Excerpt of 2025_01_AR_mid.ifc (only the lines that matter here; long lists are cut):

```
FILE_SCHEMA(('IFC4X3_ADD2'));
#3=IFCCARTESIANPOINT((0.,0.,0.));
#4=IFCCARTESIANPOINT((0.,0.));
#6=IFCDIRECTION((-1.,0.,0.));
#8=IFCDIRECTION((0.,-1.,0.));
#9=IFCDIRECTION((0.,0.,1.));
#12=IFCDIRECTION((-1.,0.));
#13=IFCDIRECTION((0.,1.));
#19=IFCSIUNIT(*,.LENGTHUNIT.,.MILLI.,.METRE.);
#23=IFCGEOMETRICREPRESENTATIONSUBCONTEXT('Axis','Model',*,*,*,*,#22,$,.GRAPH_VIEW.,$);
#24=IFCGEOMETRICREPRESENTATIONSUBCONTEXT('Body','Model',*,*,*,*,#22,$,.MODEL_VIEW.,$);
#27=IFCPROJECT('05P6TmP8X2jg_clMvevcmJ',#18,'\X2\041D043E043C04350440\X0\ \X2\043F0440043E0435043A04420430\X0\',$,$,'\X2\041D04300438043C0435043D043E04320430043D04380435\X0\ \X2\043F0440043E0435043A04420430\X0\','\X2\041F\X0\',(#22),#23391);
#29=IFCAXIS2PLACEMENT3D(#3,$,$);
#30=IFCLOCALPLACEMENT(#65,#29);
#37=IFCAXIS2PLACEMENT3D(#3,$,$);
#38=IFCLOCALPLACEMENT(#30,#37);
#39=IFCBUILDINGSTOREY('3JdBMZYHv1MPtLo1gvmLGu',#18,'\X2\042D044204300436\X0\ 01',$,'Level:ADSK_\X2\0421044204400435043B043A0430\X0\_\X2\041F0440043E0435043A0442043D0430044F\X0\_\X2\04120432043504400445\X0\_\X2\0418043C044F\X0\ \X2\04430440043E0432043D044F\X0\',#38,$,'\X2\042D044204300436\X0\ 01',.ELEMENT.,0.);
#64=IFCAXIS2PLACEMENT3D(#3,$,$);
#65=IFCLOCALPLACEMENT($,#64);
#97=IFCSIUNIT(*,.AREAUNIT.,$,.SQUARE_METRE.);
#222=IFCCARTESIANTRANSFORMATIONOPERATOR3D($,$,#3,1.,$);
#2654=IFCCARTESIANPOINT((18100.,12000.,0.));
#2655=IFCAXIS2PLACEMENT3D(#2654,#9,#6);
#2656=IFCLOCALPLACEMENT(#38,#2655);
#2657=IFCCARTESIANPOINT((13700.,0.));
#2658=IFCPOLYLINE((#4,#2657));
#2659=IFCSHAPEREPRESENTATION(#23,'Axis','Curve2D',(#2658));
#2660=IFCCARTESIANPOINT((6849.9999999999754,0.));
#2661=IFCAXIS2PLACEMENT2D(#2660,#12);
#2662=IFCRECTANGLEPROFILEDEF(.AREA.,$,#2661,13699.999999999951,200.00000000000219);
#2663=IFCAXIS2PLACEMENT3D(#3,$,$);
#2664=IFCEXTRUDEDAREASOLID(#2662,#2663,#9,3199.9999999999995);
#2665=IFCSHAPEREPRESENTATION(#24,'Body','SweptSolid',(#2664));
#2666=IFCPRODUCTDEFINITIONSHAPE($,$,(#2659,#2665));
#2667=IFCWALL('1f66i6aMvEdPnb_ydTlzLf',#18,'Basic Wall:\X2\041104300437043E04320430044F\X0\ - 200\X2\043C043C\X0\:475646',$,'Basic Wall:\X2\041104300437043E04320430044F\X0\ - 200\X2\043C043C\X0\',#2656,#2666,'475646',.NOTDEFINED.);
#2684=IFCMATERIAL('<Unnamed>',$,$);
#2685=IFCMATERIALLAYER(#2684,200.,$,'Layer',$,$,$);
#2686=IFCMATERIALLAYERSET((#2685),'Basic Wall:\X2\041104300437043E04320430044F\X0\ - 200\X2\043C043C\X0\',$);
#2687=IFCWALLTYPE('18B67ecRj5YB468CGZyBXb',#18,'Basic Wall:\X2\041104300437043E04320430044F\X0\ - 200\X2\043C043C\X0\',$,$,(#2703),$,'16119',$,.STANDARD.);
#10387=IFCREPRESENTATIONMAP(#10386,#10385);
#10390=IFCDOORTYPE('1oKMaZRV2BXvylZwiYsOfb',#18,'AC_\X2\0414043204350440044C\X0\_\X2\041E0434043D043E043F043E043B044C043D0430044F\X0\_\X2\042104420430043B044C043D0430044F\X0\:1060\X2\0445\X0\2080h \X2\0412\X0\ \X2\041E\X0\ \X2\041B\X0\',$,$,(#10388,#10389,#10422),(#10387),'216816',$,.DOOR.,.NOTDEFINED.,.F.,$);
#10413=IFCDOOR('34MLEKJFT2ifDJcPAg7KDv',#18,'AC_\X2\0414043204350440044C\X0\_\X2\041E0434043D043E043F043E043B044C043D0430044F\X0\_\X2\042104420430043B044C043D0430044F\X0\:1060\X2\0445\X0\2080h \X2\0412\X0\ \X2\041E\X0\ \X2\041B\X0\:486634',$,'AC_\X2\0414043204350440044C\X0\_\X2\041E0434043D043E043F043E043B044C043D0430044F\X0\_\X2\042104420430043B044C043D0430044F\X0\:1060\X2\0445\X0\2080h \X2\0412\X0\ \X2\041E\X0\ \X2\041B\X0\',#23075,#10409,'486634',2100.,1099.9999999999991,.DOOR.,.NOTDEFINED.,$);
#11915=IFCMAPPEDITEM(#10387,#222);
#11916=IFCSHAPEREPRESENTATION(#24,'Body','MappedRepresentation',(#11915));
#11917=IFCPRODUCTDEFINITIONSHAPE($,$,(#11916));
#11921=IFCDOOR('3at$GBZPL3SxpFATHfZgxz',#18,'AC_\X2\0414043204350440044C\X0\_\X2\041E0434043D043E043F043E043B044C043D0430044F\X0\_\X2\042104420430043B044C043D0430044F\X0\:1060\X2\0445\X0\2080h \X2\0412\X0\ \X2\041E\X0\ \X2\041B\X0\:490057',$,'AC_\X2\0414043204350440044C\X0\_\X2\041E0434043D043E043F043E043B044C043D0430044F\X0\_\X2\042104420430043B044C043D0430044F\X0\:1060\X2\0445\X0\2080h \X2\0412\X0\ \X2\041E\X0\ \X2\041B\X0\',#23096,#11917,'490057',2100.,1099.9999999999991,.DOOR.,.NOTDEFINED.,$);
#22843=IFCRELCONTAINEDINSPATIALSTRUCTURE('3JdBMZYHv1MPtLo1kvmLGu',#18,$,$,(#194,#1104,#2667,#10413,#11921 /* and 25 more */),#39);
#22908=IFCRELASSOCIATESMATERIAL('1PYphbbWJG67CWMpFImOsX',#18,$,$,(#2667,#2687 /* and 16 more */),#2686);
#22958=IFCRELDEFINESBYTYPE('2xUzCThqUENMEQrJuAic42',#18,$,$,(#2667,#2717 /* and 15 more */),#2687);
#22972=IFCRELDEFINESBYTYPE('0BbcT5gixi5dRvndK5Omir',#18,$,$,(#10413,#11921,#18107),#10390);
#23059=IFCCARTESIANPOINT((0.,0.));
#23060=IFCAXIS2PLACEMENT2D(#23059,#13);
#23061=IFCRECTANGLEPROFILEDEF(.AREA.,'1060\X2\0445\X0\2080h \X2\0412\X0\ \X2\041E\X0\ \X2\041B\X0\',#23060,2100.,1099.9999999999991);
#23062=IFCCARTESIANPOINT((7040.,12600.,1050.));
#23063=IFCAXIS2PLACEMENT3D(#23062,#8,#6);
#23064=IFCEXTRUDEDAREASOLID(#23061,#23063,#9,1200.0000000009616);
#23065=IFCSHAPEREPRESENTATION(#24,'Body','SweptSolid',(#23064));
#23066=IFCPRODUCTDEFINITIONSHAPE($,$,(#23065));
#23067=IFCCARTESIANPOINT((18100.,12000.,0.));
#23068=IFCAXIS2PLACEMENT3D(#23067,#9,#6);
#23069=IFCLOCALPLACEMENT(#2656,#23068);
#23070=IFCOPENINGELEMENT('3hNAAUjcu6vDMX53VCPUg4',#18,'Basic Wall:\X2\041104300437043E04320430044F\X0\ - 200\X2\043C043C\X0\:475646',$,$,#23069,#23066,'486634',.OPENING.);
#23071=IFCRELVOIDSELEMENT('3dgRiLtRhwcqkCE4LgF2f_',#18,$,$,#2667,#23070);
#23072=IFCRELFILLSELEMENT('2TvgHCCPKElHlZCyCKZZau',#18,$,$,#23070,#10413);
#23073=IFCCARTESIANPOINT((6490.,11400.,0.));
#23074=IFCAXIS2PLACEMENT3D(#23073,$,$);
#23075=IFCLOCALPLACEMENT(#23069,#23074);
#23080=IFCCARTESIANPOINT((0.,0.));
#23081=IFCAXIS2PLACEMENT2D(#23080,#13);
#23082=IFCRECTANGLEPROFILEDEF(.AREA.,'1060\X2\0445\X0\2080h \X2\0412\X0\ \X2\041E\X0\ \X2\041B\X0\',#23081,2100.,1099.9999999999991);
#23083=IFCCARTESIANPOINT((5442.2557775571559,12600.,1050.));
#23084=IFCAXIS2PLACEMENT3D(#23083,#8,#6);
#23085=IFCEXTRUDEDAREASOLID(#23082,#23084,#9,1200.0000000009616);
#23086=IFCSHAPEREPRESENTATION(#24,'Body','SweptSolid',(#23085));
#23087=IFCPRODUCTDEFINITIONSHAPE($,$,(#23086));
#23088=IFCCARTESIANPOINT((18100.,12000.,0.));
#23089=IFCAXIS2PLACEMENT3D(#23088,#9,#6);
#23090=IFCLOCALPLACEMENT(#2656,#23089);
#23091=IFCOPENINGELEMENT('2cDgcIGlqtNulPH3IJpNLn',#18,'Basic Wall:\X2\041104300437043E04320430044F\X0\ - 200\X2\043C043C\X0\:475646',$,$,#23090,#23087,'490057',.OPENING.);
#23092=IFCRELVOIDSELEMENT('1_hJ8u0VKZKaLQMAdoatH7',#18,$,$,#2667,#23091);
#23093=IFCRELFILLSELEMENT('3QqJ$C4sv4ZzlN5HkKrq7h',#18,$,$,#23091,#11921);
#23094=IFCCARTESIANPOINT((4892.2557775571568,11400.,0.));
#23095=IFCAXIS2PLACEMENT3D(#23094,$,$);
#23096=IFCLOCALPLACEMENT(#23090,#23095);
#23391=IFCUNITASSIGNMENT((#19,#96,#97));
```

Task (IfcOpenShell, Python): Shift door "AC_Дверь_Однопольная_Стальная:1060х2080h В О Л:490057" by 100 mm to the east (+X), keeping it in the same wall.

```python
import ifcopenshell
import ifcopenshell.api.geometry
import ifcopenshell.util.placement
import ifcopenshell.util.unit

model = ifcopenshell.open("2025_01_AR_mid.ifc")
unit_scale = ifcopenshell.util.unit.calculate_unit_scale(model)

door = model.by_guid("3at$GBZPL3SxpFATHfZgxz")
opening = door.FillsVoids[0].RelatingOpeningElement
wall = opening.VoidsElements[0].RelatingBuildingElement

wall_matrix = ifcopenshell.util.placement.get_local_placement(wall.ObjectPlacement)
shift = wall_matrix[:3, 0] * -0.1 / unit_scale
before = ifcopenshell.util.placement.get_local_placement(door.ObjectPlacement)[:3, 3].copy()

# The door is placed relative to its opening, so it follows when the opening moves.
matrix = ifcopenshell.util.placement.get_local_placement(opening.ObjectPlacement)
matrix[:3, 3] += shift
ifcopenshell.api.geometry.edit_object_placement(
    model, product=opening, matrix=matrix, is_si=False, should_transform_children=True
)

after = ifcopenshell.util.placement.get_local_placement(door.ObjectPlacement)[:3, 3]
print("door moved by", (after - before).round(3) + 0.0)

model.write("2025_01_AR_mid-out.ifc")
```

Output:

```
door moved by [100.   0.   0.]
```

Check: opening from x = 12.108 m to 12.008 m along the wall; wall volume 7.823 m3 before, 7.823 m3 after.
